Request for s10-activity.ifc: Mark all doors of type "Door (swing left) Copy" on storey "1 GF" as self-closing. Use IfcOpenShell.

First a look at what the model holds.

```python
import ifcopenshell
import ifcopenshell.util.element

model = ifcopenshell.open("s10-activity.ifc")
print(model.schema)
storey = next(s for s in model.by_type("IfcBuildingStorey") if s.Name == "1 GF")
doors = [e for e in ifcopenshell.util.element.get_decomposition(storey) if e.is_a("IfcDoor")]
seen = {}
for e in doors:
    element_type = ifcopenshell.util.element.get_type(e)
    key = (element_type.Name if element_type != e and element_type else None, ifcopenshell.util.element.get_pset(e, "Pset_DoorCommon", "SelfClosing"))
    seen[key] = seen.get(key, 0) + 1
for (name, value), count in sorted(seen.items(), key=str):
    print(count, "x", name, "|", value)
```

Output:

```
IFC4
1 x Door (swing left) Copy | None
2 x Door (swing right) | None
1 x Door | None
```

```python
import ifcopenshell
import ifcopenshell.api.pset
import ifcopenshell.util.element

model = ifcopenshell.open("s10-activity.ifc")

storey = next(s for s in model.by_type("IfcBuildingStorey") if s.Name == "1 GF")
doors = [e for e in ifcopenshell.util.element.get_decomposition(storey) if e.is_a("IfcDoor")]

count = 0
for e in doors:
    element_type = ifcopenshell.util.element.get_type(e)
    if element_type in (None, e) or element_type.Name != "Door (swing left) Copy":
        continue
    # add_pset returns the element's existing set when there is one.
    pset = ifcopenshell.api.pset.add_pset(model, product=e, name="Pset_DoorCommon")
    ifcopenshell.api.pset.edit_pset(model, pset=pset, properties={"SelfClosing": True})
    count += 1

print(count, "doors updated")

model.write("s10-activity_v2.ifc")
```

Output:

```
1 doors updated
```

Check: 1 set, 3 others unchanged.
